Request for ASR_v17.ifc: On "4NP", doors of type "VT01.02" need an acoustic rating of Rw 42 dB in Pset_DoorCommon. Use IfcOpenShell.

First a look at what the model holds.

```python
import ifcopenshell
import ifcopenshell.util.element

model = ifcopenshell.open("ASR_v17.ifc")
print(model.schema)
storey = next(s for s in model.by_type("IfcBuildingStorey") if s.Name == "4NP")
doors = [e for e in ifcopenshell.util.element.get_decomposition(storey) if e.is_a("IfcDoor")]
seen = {}
for e in doors:
    element_type = ifcopenshell.util.element.get_type(e)
    key = (element_type.Name if element_type != e and element_type else None, ifcopenshell.util.element.get_pset(e, "Pset_DoorCommon", "AcousticRating"))
    seen[key] = seen.get(key, 0) + 1
for (name, value), count in sorted(seen.items(), key=str):
    print(count, "x", name, "|", value)
```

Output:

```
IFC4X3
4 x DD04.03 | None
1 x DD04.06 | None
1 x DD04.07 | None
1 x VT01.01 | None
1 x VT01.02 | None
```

```python
import ifcopenshell
import ifcopenshell.api.pset
import ifcopenshell.util.element

model = ifcopenshell.open("ASR_v17.ifc")

storey = next(s for s in model.by_type("IfcBuildingStorey") if s.Name == "4NP")
doors = [e for e in ifcopenshell.util.element.get_decomposition(storey) if e.is_a("IfcDoor")]

count = 0
for e in doors:
    element_type = ifcopenshell.util.element.get_type(e)
    if element_type in (None, e) or element_type.Name != "VT01.02":
        continue
    # add_pset returns the element's existing set when there is one.
    pset = ifcopenshell.api.pset.add_pset(model, product=e, name="Pset_DoorCommon")
    ifcopenshell.api.pset.edit_pset(model, pset=pset, properties={"AcousticRating": "Rw 42 dB"})
    count += 1

print(count, "doors updated")

model.write("ASR_v17_edited.ifc")
```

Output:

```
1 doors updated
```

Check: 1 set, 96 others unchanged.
